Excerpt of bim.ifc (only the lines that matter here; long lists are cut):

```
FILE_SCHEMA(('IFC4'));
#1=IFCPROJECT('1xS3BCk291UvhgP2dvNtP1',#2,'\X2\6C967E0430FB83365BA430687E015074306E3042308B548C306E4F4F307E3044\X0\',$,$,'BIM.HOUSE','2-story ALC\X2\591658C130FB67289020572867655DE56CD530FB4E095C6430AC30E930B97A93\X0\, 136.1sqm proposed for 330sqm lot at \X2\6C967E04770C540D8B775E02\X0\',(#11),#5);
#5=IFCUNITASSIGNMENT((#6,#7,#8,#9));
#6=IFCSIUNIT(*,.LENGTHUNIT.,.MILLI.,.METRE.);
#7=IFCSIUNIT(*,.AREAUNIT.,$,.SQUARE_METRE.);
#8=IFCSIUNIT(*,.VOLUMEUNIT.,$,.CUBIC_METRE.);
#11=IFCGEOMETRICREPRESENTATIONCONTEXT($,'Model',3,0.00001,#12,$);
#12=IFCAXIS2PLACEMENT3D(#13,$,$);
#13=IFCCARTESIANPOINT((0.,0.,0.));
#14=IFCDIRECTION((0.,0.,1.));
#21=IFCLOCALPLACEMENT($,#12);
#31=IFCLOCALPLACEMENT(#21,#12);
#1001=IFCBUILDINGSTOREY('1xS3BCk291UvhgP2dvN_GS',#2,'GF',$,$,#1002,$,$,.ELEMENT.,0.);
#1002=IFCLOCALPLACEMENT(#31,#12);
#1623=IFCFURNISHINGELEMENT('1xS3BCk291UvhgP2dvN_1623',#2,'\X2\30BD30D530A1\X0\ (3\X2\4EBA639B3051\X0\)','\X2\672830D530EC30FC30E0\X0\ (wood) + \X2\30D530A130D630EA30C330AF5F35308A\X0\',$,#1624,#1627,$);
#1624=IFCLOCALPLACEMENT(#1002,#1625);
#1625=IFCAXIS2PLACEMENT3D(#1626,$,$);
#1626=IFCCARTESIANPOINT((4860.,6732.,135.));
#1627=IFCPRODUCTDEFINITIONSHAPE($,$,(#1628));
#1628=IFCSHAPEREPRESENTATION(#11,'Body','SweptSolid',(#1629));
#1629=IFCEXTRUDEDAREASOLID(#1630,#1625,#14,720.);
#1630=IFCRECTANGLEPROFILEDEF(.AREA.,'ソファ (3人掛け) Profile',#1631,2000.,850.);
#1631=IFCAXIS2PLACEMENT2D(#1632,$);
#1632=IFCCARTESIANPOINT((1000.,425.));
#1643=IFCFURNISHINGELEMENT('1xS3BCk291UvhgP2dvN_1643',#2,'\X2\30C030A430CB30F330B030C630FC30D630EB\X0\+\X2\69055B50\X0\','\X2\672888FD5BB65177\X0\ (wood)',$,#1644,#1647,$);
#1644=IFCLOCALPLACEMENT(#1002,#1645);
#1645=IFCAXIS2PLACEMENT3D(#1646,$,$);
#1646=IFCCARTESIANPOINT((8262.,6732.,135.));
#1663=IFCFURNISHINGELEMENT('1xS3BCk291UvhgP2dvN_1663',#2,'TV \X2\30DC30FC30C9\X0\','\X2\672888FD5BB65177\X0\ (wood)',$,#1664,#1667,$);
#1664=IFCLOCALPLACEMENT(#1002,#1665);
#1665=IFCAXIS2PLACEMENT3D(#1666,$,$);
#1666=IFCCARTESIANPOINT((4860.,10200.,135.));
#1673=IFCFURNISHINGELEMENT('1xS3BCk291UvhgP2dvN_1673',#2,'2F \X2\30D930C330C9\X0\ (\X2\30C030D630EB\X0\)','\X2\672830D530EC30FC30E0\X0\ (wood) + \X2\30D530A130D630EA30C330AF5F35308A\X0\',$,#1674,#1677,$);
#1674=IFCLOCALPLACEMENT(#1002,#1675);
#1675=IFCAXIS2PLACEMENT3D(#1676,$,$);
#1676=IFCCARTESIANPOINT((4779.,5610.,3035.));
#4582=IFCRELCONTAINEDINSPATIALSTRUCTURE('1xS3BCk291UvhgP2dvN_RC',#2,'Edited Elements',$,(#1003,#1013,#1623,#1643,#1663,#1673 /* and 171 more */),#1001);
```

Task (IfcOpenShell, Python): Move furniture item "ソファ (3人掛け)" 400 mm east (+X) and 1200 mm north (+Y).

```python
import ifcopenshell
import ifcopenshell.api.geometry
import ifcopenshell.util.placement
import ifcopenshell.util.unit

model = ifcopenshell.open("bim.ifc")
unit_scale = ifcopenshell.util.unit.calculate_unit_scale(model)

item = model.by_guid("1xS3BCk291UvhgP2dvN_1623")
matrix = ifcopenshell.util.placement.get_local_placement(item.ObjectPlacement)
matrix[0, 3] += 0.4 / unit_scale
matrix[1, 3] += 1.2 / unit_scale
ifcopenshell.api.geometry.edit_object_placement(model, product=item, matrix=matrix, is_si=False)

print(ifcopenshell.util.placement.get_local_placement(item.ObjectPlacement).round(3) + 0.0)

model.write("bim_v2.ifc")
```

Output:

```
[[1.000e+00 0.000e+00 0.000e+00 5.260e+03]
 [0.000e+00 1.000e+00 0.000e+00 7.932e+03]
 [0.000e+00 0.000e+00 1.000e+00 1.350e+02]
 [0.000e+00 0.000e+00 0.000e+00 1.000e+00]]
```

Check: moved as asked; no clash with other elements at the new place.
